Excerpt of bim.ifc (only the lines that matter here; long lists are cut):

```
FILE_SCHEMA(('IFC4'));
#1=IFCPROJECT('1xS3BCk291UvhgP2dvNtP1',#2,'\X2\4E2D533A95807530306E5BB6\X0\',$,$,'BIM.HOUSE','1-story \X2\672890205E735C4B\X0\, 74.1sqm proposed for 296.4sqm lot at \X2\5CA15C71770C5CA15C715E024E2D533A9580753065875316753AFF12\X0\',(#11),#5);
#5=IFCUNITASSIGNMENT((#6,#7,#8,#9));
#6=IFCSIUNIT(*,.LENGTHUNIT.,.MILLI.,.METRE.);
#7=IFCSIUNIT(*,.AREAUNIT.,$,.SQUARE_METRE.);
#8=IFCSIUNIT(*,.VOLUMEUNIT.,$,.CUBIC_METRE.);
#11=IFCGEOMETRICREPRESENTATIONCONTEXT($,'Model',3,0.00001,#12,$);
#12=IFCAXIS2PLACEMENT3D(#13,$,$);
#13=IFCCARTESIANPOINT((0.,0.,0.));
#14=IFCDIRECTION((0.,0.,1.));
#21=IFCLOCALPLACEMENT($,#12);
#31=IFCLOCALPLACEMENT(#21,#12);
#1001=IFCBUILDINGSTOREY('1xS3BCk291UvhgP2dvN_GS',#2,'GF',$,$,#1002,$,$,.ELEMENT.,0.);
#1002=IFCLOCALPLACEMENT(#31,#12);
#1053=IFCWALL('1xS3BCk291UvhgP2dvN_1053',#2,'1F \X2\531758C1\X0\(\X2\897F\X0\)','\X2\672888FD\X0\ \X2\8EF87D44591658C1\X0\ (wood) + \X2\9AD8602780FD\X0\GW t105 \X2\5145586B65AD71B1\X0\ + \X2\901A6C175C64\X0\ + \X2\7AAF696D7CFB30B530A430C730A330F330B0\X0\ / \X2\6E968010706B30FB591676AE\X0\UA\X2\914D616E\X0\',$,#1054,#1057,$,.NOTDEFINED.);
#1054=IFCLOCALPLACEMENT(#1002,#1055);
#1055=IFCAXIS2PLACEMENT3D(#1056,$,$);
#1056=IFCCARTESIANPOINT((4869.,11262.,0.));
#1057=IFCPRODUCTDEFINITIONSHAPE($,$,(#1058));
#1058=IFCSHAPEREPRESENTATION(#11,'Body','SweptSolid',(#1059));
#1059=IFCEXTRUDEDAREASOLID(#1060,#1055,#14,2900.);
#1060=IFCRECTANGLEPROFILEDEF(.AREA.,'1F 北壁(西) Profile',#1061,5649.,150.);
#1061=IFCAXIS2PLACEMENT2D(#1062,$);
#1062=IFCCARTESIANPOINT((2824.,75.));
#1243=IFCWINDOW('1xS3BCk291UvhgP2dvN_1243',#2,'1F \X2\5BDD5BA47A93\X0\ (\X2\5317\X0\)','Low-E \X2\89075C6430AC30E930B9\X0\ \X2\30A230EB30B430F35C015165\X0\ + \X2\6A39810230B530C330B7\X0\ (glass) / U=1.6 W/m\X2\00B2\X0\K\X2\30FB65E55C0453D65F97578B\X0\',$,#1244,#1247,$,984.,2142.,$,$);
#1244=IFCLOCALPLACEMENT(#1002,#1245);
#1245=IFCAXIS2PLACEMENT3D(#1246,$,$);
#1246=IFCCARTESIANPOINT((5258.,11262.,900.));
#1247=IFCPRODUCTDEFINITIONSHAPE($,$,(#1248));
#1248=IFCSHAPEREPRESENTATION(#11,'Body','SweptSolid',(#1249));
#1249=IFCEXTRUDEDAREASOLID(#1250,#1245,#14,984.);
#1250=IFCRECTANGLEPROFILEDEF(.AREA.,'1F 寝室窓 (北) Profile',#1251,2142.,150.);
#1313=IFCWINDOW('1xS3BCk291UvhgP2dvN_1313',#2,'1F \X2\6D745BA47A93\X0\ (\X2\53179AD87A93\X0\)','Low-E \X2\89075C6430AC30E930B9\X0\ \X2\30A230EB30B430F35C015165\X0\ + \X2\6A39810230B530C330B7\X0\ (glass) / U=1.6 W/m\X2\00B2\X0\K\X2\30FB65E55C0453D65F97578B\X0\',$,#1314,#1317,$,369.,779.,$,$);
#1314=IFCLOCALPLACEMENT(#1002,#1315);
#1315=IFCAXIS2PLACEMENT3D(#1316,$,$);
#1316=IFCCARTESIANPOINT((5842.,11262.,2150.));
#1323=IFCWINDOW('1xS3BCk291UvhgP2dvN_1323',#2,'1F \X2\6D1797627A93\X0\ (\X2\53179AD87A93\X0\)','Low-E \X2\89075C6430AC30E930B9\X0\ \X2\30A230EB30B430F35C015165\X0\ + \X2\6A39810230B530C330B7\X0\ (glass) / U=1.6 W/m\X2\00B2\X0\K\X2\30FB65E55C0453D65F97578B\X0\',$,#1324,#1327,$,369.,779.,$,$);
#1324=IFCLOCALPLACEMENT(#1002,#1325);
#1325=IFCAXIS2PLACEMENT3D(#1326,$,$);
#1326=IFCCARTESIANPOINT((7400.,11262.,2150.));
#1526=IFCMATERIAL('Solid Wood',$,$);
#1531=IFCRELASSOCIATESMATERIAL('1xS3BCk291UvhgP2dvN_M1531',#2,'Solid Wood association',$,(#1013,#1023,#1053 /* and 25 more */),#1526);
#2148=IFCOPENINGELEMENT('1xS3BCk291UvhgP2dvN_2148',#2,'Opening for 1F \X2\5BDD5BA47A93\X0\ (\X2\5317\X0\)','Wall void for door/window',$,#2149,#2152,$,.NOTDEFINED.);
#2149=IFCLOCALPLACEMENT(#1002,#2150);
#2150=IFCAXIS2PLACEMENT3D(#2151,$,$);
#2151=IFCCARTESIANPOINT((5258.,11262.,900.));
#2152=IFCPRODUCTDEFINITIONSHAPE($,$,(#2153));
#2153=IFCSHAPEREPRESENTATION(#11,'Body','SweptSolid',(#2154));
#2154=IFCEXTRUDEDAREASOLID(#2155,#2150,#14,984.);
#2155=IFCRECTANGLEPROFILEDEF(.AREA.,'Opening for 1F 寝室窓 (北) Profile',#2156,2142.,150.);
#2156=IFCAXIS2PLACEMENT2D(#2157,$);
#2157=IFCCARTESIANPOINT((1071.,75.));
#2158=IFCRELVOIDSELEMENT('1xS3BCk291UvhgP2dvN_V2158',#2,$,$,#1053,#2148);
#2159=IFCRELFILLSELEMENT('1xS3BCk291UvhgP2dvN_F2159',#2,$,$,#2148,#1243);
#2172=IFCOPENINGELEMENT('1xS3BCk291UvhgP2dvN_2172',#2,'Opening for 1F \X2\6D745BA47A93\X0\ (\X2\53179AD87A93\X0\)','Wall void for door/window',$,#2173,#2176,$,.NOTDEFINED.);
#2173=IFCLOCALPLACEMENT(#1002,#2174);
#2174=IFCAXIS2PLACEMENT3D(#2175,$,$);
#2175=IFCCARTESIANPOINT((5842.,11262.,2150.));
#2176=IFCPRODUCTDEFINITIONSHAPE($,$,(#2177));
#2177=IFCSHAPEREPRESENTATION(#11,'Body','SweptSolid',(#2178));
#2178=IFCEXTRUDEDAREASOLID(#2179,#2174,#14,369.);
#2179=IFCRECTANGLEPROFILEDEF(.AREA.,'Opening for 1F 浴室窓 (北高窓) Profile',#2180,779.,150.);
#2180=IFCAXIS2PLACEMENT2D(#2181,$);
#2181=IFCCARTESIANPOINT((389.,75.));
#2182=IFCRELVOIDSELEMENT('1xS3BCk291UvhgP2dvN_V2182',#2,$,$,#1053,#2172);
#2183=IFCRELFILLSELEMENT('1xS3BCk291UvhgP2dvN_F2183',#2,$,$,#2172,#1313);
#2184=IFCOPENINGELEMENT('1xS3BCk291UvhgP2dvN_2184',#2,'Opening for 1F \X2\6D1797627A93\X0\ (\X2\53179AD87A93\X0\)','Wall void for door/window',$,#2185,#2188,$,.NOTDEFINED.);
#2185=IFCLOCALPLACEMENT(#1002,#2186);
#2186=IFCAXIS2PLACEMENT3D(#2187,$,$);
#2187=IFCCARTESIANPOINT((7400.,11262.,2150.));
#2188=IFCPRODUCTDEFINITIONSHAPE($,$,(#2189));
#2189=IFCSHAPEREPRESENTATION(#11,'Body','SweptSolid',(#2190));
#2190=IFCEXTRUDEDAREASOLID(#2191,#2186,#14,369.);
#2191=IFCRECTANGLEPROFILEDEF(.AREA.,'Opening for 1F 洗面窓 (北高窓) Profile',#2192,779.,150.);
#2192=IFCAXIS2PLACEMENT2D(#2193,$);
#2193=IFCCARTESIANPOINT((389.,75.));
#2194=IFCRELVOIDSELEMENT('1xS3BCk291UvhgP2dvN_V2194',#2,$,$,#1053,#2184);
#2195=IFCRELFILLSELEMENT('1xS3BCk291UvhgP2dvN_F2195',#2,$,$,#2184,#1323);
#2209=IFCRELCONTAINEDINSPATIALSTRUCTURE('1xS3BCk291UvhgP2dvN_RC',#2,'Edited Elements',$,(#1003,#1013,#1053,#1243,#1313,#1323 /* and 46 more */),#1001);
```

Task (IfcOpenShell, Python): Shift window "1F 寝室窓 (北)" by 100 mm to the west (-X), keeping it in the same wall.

```python
import ifcopenshell
import ifcopenshell.api.geometry
import ifcopenshell.util.placement
import ifcopenshell.util.unit

model = ifcopenshell.open("bim.ifc")
unit_scale = ifcopenshell.util.unit.calculate_unit_scale(model)

window = model.by_guid("1xS3BCk291UvhgP2dvN_1243")
opening = window.FillsVoids[0].RelatingOpeningElement
wall = opening.VoidsElements[0].RelatingBuildingElement

wall_matrix = ifcopenshell.util.placement.get_local_placement(wall.ObjectPlacement)
shift = wall_matrix[:3, 0] * -0.1 / unit_scale
before = ifcopenshell.util.placement.get_local_placement(window.ObjectPlacement)[:3, 3].copy()

# The window is not placed relative to its opening, so move both.
for product in (opening, window):
    matrix = ifcopenshell.util.placement.get_local_placement(product.ObjectPlacement)
    matrix[:3, 3] += shift
    ifcopenshell.api.geometry.edit_object_placement(model, product=product, matrix=matrix, is_si=False)

after = ifcopenshell.util.placement.get_local_placement(window.ObjectPlacement)[:3, 3]
print("window moved by", (after - before).round(3) + 0.0)

model.write("bim_updated.ifc")
```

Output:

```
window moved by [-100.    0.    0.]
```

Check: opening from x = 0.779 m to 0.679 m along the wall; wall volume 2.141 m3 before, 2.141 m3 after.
